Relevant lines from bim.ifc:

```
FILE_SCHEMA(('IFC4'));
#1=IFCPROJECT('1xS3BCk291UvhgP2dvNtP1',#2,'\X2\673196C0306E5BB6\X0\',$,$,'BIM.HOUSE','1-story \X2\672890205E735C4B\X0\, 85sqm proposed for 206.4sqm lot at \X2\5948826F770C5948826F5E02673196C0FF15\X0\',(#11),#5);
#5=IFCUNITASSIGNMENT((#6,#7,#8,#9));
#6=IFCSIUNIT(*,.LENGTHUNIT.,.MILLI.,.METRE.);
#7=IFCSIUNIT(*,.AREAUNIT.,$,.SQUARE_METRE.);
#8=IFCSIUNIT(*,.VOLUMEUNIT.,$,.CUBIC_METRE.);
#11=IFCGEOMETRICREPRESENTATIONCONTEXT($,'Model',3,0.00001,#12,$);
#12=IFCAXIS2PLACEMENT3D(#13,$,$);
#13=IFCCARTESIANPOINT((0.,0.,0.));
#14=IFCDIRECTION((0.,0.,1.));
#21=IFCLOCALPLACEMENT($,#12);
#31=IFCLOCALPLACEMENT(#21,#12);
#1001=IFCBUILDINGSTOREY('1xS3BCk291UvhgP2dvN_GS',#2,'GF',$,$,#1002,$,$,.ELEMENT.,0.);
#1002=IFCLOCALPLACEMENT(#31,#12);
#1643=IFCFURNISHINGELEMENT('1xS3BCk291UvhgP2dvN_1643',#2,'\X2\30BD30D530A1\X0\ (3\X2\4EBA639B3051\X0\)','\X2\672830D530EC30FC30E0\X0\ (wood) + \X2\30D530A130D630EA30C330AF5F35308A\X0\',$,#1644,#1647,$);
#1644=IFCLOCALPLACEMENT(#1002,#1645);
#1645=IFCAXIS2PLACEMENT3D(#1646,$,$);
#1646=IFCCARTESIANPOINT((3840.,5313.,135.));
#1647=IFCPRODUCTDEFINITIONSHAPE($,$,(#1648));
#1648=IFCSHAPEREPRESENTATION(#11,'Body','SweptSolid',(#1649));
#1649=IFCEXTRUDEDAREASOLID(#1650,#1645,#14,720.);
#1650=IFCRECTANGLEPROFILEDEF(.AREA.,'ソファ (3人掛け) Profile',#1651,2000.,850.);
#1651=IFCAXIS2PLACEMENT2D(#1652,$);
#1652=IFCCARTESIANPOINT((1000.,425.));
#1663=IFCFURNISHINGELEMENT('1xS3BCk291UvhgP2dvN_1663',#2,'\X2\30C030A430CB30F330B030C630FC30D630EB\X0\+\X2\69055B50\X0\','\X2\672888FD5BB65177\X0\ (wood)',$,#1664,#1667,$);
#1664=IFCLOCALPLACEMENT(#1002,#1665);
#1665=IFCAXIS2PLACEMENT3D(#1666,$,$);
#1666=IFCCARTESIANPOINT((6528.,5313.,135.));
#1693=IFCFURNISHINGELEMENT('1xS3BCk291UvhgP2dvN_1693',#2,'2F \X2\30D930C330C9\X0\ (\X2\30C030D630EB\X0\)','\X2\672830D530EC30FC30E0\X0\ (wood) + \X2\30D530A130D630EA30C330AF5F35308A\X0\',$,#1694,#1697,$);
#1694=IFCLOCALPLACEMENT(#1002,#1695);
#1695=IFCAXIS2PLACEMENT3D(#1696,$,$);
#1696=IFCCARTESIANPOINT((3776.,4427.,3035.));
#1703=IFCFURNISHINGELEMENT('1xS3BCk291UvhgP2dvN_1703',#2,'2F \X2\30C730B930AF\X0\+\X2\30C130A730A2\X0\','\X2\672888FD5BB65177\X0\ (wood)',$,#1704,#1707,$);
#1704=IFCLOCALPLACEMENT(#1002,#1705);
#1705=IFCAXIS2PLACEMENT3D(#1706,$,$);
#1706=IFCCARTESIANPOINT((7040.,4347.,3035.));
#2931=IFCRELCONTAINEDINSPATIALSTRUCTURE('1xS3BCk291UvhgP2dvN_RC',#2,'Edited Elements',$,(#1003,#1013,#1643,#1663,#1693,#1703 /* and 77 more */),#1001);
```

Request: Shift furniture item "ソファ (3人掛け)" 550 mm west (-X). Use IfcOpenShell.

```python
import ifcopenshell
import ifcopenshell.api.geometry
import ifcopenshell.util.placement
import ifcopenshell.util.unit

model = ifcopenshell.open("bim.ifc")
unit_scale = ifcopenshell.util.unit.calculate_unit_scale(model)

item = model.by_id(1643)
matrix = ifcopenshell.util.placement.get_local_placement(item.ObjectPlacement)
matrix[0, 3] -= 0.55 / unit_scale
ifcopenshell.api.geometry.edit_object_placement(model, product=item, matrix=matrix, is_si=False)

print(ifcopenshell.util.placement.get_local_placement(item.ObjectPlacement).round(3) + 0.0)

model.write("bim-out.ifc")
```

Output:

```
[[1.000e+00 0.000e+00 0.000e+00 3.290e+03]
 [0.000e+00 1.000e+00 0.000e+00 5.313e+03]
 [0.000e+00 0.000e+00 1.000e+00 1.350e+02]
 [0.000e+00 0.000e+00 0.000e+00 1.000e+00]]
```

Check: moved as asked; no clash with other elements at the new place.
